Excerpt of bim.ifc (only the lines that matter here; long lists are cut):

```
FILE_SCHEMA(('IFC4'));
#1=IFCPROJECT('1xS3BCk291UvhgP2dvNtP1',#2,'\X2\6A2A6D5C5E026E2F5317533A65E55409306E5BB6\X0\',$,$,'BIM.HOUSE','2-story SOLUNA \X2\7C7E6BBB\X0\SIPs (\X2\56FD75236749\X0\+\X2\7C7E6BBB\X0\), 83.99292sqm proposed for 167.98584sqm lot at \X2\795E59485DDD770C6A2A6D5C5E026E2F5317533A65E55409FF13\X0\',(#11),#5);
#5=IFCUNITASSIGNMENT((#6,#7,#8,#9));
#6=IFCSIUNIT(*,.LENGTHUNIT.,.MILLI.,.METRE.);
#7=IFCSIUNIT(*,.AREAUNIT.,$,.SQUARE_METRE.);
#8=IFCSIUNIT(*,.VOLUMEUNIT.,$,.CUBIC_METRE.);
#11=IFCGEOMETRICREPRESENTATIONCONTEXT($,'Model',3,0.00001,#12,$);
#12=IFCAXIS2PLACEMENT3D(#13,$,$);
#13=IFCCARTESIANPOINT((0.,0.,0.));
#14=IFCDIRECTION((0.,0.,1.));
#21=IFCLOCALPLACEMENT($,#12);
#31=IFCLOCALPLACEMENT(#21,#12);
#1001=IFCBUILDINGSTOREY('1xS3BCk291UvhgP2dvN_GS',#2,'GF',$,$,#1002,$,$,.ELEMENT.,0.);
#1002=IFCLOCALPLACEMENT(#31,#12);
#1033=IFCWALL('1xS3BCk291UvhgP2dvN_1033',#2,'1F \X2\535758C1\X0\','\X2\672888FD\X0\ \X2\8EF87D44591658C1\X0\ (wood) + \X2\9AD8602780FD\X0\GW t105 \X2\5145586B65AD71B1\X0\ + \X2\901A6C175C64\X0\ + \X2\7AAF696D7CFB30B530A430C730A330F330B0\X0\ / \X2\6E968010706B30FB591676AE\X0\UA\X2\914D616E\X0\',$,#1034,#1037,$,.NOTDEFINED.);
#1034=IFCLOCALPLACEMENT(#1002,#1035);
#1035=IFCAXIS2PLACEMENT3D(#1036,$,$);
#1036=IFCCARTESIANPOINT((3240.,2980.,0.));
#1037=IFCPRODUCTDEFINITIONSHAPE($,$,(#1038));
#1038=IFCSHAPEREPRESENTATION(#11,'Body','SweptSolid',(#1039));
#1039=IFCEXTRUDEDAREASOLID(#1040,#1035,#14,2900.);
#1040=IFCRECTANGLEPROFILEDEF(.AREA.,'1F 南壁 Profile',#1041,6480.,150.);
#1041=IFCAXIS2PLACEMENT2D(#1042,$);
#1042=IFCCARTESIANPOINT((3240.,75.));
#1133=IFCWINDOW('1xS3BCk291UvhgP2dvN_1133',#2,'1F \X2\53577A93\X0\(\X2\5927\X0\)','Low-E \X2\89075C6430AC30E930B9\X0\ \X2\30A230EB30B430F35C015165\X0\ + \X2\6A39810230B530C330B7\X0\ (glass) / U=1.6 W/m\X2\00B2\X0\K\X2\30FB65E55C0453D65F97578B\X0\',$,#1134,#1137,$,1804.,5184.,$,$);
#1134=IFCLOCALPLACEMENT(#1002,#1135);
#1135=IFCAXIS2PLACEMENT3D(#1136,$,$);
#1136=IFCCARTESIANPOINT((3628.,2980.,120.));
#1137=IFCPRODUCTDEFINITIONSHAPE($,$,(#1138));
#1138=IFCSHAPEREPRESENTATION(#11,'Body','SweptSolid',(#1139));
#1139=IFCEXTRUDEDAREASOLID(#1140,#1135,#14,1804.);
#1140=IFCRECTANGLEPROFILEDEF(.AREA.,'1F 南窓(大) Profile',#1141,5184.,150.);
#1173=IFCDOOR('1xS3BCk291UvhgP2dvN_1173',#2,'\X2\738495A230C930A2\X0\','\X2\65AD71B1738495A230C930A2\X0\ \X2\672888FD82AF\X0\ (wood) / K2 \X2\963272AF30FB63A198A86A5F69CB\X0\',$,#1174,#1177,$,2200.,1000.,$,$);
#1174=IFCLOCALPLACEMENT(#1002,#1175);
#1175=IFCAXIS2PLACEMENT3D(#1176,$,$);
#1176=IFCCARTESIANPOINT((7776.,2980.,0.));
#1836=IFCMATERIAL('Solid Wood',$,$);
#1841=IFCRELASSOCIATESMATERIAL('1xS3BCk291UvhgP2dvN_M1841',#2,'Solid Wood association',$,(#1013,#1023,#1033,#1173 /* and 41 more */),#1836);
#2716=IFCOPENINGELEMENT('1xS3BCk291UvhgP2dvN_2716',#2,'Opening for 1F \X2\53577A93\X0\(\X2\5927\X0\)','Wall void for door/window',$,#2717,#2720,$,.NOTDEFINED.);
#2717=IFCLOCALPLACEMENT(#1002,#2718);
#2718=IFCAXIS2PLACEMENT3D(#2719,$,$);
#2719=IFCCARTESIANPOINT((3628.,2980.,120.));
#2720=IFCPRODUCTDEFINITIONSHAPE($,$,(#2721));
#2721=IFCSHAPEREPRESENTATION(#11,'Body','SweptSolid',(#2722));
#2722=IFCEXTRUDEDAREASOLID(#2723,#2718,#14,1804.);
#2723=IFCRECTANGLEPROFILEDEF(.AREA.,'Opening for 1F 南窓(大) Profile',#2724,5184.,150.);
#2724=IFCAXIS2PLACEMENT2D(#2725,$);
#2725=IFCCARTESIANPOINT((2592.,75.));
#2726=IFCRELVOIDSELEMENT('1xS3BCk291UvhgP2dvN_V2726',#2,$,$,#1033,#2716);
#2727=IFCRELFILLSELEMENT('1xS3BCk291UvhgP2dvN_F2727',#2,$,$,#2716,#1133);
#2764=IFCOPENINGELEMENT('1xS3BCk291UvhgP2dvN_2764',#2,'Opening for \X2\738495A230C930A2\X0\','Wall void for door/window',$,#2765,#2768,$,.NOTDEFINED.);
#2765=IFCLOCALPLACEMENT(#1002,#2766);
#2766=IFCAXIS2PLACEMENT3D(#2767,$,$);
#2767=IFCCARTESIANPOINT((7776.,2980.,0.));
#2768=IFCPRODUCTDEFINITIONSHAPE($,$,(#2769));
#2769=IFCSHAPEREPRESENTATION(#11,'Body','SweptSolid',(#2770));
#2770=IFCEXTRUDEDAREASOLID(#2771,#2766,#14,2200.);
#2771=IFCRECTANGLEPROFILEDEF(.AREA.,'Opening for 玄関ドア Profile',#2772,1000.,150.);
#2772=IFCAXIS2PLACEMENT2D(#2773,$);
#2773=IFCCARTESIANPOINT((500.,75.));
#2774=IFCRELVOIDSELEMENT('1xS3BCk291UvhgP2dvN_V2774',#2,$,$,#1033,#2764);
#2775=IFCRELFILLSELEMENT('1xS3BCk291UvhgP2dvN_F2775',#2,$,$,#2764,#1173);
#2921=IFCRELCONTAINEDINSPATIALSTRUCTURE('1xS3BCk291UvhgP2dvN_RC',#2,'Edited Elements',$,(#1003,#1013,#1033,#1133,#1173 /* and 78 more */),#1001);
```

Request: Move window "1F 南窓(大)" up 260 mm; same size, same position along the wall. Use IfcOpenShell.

```python
import numpy as np
import ifcopenshell
import ifcopenshell.api.geometry
import ifcopenshell.util.placement
import ifcopenshell.util.unit

model = ifcopenshell.open("bim.ifc")
unit_scale = ifcopenshell.util.unit.calculate_unit_scale(model)

window = model.by_id(1133)
opening = window.FillsVoids[0].RelatingOpeningElement
dz = 0.26 / unit_scale

shift = np.array([0.0, 0.0, dz])
# The window is not placed relative to its opening, so move both.
for product in (opening, window):
    matrix = ifcopenshell.util.placement.get_local_placement(product.ObjectPlacement)
    matrix[:3, 3] += shift
    ifcopenshell.api.geometry.edit_object_placement(model, product=product, matrix=matrix, is_si=False)

print(f"moved by {dz * unit_scale:+.3f} m")

model.write("bim_edited.ifc")
```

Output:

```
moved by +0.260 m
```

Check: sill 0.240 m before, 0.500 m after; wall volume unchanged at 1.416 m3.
